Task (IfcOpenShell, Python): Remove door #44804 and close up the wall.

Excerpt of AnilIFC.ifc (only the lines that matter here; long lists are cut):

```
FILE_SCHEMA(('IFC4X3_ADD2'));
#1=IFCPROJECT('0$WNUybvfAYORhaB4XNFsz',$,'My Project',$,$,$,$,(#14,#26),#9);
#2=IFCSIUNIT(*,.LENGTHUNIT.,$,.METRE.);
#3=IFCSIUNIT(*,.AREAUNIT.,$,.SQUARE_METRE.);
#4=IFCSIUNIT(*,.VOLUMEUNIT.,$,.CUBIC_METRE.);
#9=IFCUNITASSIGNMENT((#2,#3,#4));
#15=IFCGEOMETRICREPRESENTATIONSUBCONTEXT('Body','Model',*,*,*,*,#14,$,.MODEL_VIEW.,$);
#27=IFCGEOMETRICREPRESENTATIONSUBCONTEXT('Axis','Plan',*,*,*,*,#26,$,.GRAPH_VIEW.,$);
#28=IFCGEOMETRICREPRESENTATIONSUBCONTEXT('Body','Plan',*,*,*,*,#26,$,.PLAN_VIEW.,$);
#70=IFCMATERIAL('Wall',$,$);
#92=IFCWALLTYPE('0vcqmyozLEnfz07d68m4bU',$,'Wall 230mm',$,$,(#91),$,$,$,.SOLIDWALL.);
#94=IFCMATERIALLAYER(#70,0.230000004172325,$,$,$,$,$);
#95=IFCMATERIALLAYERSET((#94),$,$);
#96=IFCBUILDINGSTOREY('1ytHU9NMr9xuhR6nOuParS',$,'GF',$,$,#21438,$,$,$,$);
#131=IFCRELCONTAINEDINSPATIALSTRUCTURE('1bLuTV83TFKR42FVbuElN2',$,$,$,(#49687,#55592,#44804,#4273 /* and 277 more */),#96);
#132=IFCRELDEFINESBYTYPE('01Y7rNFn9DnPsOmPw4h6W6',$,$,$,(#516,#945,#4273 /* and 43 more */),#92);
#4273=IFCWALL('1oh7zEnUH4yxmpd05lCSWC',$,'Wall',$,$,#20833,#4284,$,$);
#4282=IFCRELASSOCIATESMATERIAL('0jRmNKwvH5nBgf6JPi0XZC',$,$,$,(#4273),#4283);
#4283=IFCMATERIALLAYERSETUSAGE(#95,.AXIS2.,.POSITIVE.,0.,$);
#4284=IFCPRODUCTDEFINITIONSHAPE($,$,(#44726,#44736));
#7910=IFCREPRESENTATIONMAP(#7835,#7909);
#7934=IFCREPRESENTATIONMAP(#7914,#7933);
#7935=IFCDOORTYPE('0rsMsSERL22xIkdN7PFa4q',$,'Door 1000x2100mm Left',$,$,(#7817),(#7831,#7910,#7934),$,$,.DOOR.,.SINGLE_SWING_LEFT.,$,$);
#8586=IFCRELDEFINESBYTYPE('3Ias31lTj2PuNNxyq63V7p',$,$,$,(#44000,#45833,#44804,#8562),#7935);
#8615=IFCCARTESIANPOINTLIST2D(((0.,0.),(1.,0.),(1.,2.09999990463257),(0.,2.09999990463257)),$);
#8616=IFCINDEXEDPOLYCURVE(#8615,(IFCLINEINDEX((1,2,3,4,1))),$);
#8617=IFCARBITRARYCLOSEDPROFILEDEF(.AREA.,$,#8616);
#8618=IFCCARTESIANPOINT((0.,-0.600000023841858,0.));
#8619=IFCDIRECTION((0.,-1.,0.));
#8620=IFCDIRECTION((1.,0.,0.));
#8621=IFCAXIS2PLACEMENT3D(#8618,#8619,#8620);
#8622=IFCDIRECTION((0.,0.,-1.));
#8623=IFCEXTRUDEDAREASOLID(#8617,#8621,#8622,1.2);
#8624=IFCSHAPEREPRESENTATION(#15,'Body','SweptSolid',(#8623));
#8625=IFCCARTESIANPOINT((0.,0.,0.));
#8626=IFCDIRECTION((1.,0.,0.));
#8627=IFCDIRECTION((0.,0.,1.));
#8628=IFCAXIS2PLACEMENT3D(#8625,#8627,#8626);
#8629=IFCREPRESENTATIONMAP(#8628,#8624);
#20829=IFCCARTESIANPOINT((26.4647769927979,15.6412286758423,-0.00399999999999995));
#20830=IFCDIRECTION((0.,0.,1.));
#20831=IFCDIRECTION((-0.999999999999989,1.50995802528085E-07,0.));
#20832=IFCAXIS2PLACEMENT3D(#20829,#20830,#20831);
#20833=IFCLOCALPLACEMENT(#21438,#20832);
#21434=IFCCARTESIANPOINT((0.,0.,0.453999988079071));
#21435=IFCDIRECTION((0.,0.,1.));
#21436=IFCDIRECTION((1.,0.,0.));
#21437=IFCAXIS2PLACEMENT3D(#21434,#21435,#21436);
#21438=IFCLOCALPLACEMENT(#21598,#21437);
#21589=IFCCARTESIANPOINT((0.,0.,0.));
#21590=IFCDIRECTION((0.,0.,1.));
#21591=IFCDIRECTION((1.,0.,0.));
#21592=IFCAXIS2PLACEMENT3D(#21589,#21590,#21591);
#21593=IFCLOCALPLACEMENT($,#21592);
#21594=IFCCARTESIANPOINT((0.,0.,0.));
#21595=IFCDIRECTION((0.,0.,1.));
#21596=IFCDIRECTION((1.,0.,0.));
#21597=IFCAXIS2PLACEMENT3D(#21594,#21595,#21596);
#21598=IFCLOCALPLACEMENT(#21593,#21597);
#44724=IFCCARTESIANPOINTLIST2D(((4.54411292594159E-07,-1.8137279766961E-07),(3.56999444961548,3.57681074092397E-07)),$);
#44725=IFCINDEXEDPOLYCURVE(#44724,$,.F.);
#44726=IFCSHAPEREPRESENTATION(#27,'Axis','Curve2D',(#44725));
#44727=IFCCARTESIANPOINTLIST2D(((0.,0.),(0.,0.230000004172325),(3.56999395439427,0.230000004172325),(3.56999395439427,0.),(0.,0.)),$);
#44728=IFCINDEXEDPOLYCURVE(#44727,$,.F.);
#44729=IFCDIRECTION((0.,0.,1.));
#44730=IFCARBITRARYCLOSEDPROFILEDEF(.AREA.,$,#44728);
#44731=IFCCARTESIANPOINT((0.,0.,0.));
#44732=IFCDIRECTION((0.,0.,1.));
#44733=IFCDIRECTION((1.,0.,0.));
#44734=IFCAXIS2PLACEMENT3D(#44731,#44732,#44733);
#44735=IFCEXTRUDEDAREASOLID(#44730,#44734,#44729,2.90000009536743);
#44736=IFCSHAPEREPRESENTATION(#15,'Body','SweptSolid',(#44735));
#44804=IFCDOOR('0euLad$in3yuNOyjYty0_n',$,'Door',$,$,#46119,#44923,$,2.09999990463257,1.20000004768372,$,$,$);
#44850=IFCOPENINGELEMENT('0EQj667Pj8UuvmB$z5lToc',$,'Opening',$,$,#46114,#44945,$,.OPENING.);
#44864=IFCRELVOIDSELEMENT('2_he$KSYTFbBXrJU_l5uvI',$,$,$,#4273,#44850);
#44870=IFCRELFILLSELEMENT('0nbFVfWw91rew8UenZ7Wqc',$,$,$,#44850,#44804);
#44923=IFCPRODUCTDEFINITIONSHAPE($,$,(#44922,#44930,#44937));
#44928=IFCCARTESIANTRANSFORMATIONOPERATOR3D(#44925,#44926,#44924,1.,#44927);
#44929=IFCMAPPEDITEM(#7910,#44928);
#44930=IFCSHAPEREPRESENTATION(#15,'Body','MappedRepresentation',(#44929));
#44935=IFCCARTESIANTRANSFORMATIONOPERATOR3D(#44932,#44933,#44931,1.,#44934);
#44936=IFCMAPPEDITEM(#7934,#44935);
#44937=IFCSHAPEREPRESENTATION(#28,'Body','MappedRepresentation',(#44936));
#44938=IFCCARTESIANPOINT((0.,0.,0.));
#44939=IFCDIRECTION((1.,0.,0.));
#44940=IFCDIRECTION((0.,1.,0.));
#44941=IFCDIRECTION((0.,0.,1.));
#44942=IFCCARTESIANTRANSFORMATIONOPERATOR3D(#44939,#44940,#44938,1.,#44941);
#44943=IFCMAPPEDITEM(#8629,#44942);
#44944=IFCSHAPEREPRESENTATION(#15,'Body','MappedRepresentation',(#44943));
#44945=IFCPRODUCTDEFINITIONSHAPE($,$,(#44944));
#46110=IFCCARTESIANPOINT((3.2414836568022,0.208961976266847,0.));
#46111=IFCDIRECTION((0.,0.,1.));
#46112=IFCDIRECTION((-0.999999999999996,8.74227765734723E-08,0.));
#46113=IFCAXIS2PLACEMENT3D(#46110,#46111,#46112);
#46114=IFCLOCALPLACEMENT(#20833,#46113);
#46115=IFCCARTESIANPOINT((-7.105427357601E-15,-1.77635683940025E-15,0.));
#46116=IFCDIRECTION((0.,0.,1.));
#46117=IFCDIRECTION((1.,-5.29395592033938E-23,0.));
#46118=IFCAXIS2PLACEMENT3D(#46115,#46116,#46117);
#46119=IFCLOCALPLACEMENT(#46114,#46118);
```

```python
import ifcopenshell
import ifcopenshell.api.feature
import ifcopenshell.api.root
import ifcopenshell.geom
import ifcopenshell.util.shape

model = ifcopenshell.open("AnilIFC.ifc")
settings = ifcopenshell.geom.settings()


def volume(element):
    """Net volume in cubic metres, openings subtracted."""
    shape = ifcopenshell.geom.create_shape(settings, element)
    return ifcopenshell.util.shape.get_volume(shape.geometry)


door = model.by_guid("0euLad$in3yuNOyjYty0_n")
opening = door.FillsVoids[0].RelatingOpeningElement
wall = opening.VoidsElements[0].RelatingBuildingElement
before = volume(wall)

ifcopenshell.api.root.remove_product(model, product=door)
ifcopenshell.api.feature.remove_feature(model, feature=opening)

after = volume(wall)

print(f"wall volume {before:.3f} -> {after:.3f} m3")

model.write("AnilIFC_v2.ifc")
```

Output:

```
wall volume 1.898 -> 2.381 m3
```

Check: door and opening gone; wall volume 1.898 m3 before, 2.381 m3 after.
